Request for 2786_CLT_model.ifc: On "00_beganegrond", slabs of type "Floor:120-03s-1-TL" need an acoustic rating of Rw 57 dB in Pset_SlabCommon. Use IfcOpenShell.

First a look at what the model holds.

```python
import ifcopenshell
import ifcopenshell.util.element

model = ifcopenshell.open("2786_CLT_model.ifc")
print(model.schema)
storey = next(s for s in model.by_type("IfcBuildingStorey") if s.Name == "00_beganegrond")
slabs = [e for e in ifcopenshell.util.element.get_decomposition(storey) if e.is_a("IfcSlab")]
seen = {}
for e in slabs:
    element_type = ifcopenshell.util.element.get_type(e)
    key = (element_type.Name if element_type != e and element_type else None, ifcopenshell.util.element.get_pset(e, "Pset_SlabCommon", "AcousticRating"))
    seen[key] = seen.get(key, 0) + 1
for (name, value), count in sorted(seen.items(), key=str):
    print(count, "x", name, "|", value)
```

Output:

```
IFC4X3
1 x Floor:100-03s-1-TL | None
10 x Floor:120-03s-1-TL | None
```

```python
import ifcopenshell
import ifcopenshell.api.pset
import ifcopenshell.util.element

model = ifcopenshell.open("2786_CLT_model.ifc")

storey = next(s for s in model.by_type("IfcBuildingStorey") if s.Name == "00_beganegrond")
slabs = [e for e in ifcopenshell.util.element.get_decomposition(storey) if e.is_a("IfcSlab")]

count = 0
for e in slabs:
    element_type = ifcopenshell.util.element.get_type(e)
    if element_type in (None, e) or element_type.Name != "Floor:120-03s-1-TL":
        continue
    # add_pset returns the element's existing set when there is one.
    pset = ifcopenshell.api.pset.add_pset(model, product=e, name="Pset_SlabCommon")
    ifcopenshell.api.pset.edit_pset(model, pset=pset, properties={"AcousticRating": "Rw 57 dB"})
    count += 1

print(count, "slabs updated")

model.write("2786_CLT_model_rev.ifc")
```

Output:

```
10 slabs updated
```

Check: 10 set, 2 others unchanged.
